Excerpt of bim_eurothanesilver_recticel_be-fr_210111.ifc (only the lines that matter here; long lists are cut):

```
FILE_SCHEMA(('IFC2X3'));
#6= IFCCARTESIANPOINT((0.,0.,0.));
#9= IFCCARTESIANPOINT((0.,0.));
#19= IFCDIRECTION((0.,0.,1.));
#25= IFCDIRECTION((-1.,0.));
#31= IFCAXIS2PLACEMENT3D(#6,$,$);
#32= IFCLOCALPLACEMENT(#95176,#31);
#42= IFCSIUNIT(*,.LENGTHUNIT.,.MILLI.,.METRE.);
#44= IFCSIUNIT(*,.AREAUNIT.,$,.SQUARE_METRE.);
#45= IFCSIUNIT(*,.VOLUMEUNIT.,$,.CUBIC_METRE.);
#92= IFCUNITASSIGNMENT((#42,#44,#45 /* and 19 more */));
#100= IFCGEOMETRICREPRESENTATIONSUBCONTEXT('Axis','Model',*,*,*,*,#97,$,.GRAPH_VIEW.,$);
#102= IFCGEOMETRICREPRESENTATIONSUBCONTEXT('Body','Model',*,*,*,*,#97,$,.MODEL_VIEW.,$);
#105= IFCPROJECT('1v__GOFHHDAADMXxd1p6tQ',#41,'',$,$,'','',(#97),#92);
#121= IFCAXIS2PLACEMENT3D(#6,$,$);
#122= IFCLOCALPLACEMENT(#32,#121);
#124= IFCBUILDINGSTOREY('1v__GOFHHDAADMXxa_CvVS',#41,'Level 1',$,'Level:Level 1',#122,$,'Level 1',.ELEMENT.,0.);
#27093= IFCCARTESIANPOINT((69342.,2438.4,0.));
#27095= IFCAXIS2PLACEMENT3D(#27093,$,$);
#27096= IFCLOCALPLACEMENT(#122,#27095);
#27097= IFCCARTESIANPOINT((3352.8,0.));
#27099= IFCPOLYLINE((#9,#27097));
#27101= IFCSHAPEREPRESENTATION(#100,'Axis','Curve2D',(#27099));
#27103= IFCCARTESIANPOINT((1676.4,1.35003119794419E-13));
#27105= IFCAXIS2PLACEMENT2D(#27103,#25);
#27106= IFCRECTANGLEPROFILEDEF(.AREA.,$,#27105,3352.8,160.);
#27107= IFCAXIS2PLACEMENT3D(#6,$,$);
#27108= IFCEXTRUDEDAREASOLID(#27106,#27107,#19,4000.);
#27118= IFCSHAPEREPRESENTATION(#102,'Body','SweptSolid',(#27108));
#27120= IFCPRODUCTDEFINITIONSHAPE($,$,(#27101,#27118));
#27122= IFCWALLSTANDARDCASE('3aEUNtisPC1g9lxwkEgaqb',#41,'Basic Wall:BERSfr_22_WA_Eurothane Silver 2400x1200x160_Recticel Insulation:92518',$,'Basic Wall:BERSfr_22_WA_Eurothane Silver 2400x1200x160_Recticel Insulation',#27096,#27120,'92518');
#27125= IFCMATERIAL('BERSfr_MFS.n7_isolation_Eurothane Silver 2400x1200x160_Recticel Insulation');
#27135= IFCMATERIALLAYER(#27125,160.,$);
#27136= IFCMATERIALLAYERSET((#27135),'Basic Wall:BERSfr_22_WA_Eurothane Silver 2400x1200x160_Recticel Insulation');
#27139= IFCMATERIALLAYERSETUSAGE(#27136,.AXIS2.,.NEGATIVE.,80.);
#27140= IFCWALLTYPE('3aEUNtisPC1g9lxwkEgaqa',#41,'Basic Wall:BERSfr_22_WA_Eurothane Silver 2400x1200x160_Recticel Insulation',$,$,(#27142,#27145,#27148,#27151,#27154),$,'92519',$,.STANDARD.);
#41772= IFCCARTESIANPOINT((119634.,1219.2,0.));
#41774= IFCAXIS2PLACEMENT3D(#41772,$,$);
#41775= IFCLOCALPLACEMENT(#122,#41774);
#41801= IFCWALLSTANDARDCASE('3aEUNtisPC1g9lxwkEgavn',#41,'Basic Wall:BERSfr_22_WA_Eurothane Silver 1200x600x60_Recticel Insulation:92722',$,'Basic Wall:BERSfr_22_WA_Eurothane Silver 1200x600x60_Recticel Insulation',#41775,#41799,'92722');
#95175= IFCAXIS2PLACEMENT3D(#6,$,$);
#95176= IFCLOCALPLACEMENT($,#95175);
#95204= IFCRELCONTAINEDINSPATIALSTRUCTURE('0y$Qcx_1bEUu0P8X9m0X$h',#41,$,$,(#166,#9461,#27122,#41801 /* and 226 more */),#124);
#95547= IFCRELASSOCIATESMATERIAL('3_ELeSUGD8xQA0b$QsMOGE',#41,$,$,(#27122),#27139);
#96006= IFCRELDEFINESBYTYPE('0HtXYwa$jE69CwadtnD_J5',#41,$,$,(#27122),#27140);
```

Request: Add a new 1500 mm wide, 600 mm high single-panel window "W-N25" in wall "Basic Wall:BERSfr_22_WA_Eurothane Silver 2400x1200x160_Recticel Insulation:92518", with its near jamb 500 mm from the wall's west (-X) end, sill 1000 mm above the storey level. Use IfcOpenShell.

```python
import numpy as np
import ifcopenshell
import ifcopenshell.api.feature
import ifcopenshell.api.geometry
import ifcopenshell.api.root
import ifcopenshell.api.spatial
import ifcopenshell.api.type
import ifcopenshell.geom
import ifcopenshell.util.element
import ifcopenshell.util.placement
import ifcopenshell.util.representation
import ifcopenshell.util.shape
import ifcopenshell.util.unit

model = ifcopenshell.open("bim_eurothanesilver_recticel_be-fr_210111.ifc")
unit_scale = ifcopenshell.util.unit.calculate_unit_scale(model)
settings = ifcopenshell.geom.settings()


def volume(element):
    """Net volume in cubic metres, openings subtracted."""
    shape = ifcopenshell.geom.create_shape(settings, element)
    return ifcopenshell.util.shape.get_volume(shape.geometry)


wall = model.by_guid("3aEUNtisPC1g9lxwkEgaqb")
storey = ifcopenshell.util.element.get_container(wall, ifc_class="IfcBuildingStorey")
context = ifcopenshell.util.representation.get_context(model, "Model", "Body", "MODEL_VIEW")
before = volume(wall)

width, height, from_end, sill = 1.5, 0.6, 0.5, 1  # metres

# The wall runs along its own X axis, and the end named is its -X end.
wall_shape = ifcopenshell.geom.create_shape(settings, wall)
x, y, z = ifcopenshell.util.shape.get_vertices(wall_shape.geometry).T
start = x.min() + from_end
face, thickness = float(y.min()), float(y.max() - y.min())
wall_matrix = ifcopenshell.util.placement.get_local_placement(wall.ObjectPlacement)
level = ifcopenshell.util.placement.get_local_placement(storey.ObjectPlacement)[2, 3]


def in_wall(x, y):
    """Placement at x, y metres in the wall's axes, at sill height."""
    matrix = wall_matrix.copy()
    matrix[:, 3] = wall_matrix @ np.array([x / unit_scale, y / unit_scale, 0.0, 1.0])
    matrix[2, 3] = level + sill / unit_scale
    return matrix


# Opening: a box that overshoots both wall faces by 50 mm.
opening = ifcopenshell.api.root.create_entity(model, ifc_class="IfcOpeningElement")
box = ifcopenshell.api.geometry.add_wall_representation(
    model, context=context, length=width, height=height, thickness=thickness + 0.1
)
ifcopenshell.api.geometry.assign_representation(model, product=opening, representation=box)
ifcopenshell.api.geometry.edit_object_placement(model, product=opening, matrix=in_wall(start, face - 0.05), is_si=False)
ifcopenshell.api.feature.add_feature(model, feature=opening, element=wall)

window = ifcopenshell.api.root.create_entity(model, ifc_class="IfcWindow", name="W-N25")
window.OverallWidth, window.OverallHeight = width / unit_scale, height / unit_scale
body = ifcopenshell.api.geometry.add_window_representation(
    model,
    context=context,
    overall_width=window.OverallWidth,
    overall_height=window.OverallHeight,
    partition_type="SINGLE_PANEL",
)
ifcopenshell.api.geometry.assign_representation(model, product=window, representation=body)
ifcopenshell.api.spatial.assign_container(model, products=[window], relating_structure=storey)
fills = ifcopenshell.api.feature.add_filling(model, opening=opening, element=window)
fills.OwnerHistory = window.OwnerHistory  # required in IFC2X3

# IFC2X3 keeps the operation on the window style.
style = ifcopenshell.api.root.create_entity(model, ifc_class="IfcWindowStyle", name="W-N25")
style.OperationType, style.ConstructionType = "SINGLE_PANEL", "NOTDEFINED"
style.ParameterTakesPrecedence = style.Sizeable = False
ifcopenshell.api.type.assign_type(model, related_objects=[window], relating_type=style)

# Centre the window in the wall's thickness.
ifcopenshell.api.geometry.edit_object_placement(model, product=window, matrix=in_wall(start, face), is_si=False)
window_shape = ifcopenshell.geom.create_shape(settings, window)
depth = ifcopenshell.util.shape.get_vertices(window_shape.geometry)[:, 1]
offset = face + thickness / 2 - (depth.min() + depth.max()) / 2
ifcopenshell.api.geometry.edit_object_placement(model, product=window, matrix=in_wall(start, offset), is_si=False)

after = volume(wall)

print(f"wall volume {before:.3f} -> {after:.3f} m3")

model.write("bim_eurothanesilver_recticel_be-fr_210111-out.ifc")
```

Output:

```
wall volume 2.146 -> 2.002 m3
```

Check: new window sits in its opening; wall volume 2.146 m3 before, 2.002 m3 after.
